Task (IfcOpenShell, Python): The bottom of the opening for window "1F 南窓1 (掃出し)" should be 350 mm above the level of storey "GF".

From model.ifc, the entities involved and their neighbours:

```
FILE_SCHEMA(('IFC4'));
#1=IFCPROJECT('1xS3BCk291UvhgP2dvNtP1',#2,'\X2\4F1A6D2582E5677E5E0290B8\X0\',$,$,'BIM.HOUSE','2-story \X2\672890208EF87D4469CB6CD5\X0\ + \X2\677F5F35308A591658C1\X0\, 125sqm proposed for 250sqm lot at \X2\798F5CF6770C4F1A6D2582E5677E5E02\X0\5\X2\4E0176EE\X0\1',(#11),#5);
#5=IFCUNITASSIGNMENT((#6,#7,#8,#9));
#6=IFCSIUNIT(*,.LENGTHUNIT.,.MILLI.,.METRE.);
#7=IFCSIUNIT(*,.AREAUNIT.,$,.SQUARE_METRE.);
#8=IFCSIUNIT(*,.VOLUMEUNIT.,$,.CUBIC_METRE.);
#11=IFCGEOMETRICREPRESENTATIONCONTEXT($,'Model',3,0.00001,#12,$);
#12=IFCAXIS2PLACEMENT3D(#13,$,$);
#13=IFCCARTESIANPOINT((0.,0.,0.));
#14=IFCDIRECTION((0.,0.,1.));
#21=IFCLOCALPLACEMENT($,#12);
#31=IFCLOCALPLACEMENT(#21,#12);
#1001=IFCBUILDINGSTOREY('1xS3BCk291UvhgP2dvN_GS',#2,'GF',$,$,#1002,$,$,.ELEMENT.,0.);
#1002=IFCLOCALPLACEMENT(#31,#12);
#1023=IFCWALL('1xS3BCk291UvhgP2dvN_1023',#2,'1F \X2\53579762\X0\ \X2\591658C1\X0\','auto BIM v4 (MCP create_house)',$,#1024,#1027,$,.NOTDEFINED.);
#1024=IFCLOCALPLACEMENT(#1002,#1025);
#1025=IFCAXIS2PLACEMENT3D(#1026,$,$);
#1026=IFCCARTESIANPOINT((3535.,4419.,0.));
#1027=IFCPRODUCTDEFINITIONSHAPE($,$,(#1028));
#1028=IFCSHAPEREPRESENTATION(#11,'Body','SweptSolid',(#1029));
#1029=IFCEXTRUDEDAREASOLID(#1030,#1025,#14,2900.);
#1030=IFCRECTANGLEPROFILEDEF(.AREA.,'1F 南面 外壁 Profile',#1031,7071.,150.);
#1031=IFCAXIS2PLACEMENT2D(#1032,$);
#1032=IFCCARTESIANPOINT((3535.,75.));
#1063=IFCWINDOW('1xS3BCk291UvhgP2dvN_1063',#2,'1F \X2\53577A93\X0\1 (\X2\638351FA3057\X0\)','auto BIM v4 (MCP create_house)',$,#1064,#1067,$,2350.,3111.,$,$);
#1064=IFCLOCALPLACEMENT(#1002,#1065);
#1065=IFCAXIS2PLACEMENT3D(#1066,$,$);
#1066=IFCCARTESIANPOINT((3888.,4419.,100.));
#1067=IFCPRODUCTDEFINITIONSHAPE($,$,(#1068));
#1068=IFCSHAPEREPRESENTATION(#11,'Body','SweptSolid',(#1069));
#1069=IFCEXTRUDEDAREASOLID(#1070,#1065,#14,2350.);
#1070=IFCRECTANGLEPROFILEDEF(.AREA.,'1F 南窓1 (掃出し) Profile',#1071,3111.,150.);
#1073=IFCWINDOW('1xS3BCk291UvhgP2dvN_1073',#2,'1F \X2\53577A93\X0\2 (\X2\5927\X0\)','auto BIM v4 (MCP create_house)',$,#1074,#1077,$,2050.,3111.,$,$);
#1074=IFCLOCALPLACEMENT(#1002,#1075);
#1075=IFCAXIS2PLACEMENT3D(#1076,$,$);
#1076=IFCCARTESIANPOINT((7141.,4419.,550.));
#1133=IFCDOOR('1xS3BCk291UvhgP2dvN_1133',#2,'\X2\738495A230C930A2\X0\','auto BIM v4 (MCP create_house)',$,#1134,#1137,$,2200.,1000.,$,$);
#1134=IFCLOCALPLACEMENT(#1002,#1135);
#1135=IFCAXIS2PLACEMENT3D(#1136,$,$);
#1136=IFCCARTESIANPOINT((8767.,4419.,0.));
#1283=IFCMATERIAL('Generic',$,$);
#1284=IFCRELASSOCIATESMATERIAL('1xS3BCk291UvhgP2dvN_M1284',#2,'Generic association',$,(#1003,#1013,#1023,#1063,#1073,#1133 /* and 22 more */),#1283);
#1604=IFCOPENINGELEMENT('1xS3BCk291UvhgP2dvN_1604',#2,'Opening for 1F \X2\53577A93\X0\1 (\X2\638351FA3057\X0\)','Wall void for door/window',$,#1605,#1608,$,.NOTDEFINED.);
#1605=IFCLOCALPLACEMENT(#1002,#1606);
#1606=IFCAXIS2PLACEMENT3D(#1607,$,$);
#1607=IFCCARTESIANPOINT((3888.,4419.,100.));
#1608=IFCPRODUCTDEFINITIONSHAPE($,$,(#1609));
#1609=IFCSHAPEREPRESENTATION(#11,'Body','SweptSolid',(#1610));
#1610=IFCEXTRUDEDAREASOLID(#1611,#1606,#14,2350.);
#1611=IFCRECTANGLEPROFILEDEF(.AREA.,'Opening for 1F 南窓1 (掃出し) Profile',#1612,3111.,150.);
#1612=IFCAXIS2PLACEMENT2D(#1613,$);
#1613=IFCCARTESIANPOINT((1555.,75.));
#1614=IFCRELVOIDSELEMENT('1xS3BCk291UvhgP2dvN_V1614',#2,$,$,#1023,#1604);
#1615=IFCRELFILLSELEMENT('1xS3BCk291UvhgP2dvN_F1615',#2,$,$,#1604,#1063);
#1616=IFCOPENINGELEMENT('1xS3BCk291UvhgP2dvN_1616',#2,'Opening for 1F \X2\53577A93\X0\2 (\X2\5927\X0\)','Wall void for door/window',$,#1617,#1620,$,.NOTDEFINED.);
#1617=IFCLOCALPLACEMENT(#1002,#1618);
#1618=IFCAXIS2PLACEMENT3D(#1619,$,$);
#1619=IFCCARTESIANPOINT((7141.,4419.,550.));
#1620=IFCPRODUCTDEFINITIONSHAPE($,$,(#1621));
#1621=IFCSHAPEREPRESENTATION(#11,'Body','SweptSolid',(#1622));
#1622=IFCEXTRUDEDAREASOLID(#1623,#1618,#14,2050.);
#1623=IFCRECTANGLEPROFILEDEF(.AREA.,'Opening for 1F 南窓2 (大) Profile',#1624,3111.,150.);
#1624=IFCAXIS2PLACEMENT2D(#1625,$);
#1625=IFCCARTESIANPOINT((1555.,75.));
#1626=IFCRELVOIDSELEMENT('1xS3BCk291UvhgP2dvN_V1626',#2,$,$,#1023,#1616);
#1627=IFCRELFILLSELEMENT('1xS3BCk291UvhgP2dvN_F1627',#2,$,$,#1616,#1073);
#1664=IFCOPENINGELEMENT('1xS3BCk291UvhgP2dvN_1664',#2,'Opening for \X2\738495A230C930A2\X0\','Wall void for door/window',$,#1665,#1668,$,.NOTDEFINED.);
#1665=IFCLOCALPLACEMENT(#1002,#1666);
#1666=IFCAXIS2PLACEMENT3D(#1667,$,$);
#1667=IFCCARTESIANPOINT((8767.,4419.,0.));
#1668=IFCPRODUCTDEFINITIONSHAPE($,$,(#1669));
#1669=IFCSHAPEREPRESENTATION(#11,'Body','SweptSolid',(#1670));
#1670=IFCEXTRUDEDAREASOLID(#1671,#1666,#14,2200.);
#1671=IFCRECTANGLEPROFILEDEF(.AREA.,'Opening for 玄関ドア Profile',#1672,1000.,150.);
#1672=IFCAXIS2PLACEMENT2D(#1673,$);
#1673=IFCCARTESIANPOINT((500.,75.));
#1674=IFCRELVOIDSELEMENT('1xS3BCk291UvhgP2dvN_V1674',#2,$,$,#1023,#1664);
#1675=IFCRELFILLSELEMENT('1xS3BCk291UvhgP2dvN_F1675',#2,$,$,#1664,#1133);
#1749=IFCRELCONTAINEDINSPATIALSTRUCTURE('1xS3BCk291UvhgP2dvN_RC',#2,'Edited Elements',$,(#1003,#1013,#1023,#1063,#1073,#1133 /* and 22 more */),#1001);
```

```python
import numpy as np
import ifcopenshell
import ifcopenshell.api.geometry
import ifcopenshell.geom
import ifcopenshell.util.element
import ifcopenshell.util.placement
import ifcopenshell.util.shape
import ifcopenshell.util.unit

model = ifcopenshell.open("model.ifc")
unit_scale = ifcopenshell.util.unit.calculate_unit_scale(model)

window = model.by_id(1063)
opening = window.FillsVoids[0].RelatingOpeningElement
storey = ifcopenshell.util.element.get_container(window, ifc_class="IfcBuildingStorey")
level = ifcopenshell.util.placement.get_local_placement(storey.ObjectPlacement)[2, 3]

# The opening's origin need not be at the sill, so measure its lowest point.
shape = ifcopenshell.geom.create_shape(ifcopenshell.geom.settings(), opening)
bottom = ifcopenshell.util.shape.get_shape_bottom_elevation(shape, shape.geometry) / unit_scale
dz = level + 0.35 / unit_scale - bottom

shift = np.array([0.0, 0.0, dz])
# The window is not placed relative to its opening, so move both.
for product in (opening, window):
    matrix = ifcopenshell.util.placement.get_local_placement(product.ObjectPlacement)
    matrix[:3, 3] += shift
    ifcopenshell.api.geometry.edit_object_placement(model, product=product, matrix=matrix, is_si=False)

print(f"moved by {dz * unit_scale:+.3f} m")

model.write("model_edited.ifc")
```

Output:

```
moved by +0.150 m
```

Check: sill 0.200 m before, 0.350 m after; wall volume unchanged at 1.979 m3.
